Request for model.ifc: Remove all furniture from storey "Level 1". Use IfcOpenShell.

First a look at what the model holds.

```python
import ifcopenshell
import ifcopenshell.util.element

model = ifcopenshell.open("model.ifc")
print(model.schema)
storey = next(s for s in model.by_type("IfcBuildingStorey") if s.Name == "Level 1")
furniture = [e for e in ifcopenshell.util.element.get_decomposition(storey) if e.is_a("IfcFurnishingElement")]
seen = {}
for e in furniture:
    element_type = ifcopenshell.util.element.get_type(e)
    name = element_type.Name if element_type not in (None, e) else None
    seen[name] = seen.get(name, 0) + 1
for name, count in sorted(seen.items(), key=str):
    print(count, "x", name)
```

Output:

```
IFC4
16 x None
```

```python
import ifcopenshell
import ifcopenshell.api.root
import ifcopenshell.util.element

model = ifcopenshell.open("model.ifc")

storey = next(s for s in model.by_type("IfcBuildingStorey") if s.Name == "Level 1")
furniture = [e for e in ifcopenshell.util.element.get_decomposition(storey) if e.is_a("IfcFurnishingElement")]

for e in furniture:
    ifcopenshell.api.root.remove_product(model, product=e)
print(len(furniture), "removed")

model.write("model_updated.ifc")
```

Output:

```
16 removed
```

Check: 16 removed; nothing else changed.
